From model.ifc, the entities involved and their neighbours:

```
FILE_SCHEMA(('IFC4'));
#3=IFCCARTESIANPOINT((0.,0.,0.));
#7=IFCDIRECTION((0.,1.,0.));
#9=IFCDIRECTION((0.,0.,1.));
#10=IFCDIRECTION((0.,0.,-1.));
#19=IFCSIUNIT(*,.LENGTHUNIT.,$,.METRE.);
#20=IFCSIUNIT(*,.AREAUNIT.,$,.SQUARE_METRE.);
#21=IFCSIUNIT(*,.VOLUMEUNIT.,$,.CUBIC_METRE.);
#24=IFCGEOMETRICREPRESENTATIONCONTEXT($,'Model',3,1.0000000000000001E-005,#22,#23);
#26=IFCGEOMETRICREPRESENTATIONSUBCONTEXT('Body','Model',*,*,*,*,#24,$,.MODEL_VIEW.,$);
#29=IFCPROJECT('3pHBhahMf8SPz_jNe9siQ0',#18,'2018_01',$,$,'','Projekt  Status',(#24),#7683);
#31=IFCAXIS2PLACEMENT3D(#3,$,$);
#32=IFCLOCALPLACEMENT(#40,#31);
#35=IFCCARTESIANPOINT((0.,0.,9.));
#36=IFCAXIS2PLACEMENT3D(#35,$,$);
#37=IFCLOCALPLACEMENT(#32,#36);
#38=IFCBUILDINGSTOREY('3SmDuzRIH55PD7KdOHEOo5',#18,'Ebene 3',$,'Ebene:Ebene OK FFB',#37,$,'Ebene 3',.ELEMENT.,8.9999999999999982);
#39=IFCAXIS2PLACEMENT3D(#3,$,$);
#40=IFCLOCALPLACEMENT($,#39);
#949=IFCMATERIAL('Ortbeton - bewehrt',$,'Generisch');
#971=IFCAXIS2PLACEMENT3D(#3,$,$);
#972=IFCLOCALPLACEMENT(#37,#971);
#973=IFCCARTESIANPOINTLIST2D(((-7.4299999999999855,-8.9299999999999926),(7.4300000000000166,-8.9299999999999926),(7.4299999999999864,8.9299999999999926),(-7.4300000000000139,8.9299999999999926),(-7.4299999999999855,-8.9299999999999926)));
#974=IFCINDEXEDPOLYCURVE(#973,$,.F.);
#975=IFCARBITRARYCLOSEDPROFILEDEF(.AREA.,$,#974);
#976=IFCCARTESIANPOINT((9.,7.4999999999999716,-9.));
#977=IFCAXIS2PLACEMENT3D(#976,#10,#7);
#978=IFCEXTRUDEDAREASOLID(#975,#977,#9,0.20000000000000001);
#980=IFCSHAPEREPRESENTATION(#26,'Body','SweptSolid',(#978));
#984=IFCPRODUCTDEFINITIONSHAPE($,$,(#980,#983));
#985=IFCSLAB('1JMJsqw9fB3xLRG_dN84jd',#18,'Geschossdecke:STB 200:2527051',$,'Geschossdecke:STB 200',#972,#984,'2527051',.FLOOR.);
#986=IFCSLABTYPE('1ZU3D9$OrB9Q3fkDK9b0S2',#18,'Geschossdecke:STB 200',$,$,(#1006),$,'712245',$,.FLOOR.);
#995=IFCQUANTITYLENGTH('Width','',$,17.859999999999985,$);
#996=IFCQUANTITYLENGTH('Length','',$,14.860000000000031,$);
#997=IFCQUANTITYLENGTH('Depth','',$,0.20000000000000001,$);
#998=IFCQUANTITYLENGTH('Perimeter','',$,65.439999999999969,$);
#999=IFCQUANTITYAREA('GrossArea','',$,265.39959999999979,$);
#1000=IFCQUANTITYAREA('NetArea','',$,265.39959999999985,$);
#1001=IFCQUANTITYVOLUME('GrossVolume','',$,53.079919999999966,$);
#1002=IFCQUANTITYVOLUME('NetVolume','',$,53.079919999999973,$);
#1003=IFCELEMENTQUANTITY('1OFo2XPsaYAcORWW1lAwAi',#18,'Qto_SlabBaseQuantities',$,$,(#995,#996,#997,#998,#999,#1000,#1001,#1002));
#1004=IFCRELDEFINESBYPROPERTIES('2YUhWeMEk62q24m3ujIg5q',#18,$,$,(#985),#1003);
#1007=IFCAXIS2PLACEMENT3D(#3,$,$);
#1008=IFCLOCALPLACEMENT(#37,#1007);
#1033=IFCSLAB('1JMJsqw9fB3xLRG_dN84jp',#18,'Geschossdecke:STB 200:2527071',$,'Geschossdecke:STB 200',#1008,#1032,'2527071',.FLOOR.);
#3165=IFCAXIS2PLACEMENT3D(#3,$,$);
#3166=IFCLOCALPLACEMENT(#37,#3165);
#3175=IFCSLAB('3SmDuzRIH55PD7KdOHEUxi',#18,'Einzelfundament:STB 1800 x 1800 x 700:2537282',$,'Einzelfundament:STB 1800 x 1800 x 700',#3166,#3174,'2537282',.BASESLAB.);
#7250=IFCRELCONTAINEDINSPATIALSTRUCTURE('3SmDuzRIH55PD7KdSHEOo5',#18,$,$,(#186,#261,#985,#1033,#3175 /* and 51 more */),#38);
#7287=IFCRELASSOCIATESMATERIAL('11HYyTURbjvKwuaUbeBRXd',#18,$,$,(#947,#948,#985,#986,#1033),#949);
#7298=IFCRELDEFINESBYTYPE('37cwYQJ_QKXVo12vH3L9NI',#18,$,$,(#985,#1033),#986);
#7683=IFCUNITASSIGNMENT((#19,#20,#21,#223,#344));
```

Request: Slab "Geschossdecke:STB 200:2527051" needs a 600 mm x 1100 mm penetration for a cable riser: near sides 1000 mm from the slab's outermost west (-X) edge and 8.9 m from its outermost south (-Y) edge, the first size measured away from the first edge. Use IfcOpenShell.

```python
import numpy as np
import ifcopenshell
import ifcopenshell.api.feature
import ifcopenshell.api.geometry
import ifcopenshell.api.pset
import ifcopenshell.api.root
import ifcopenshell.geom
import ifcopenshell.util.element
import ifcopenshell.util.placement
import ifcopenshell.util.representation
import ifcopenshell.util.shape
import ifcopenshell.util.unit

model = ifcopenshell.open("model.ifc")
unit_scale = ifcopenshell.util.unit.calculate_unit_scale(model)
area_scale = ifcopenshell.util.unit.calculate_unit_scale(model, "AREAUNIT")
volume_scale = ifcopenshell.util.unit.calculate_unit_scale(model, "VOLUMEUNIT")
settings = ifcopenshell.geom.settings()


def volume(element):
    """Net volume in cubic metres, openings subtracted."""
    shape = ifcopenshell.geom.create_shape(settings, element)
    return ifcopenshell.util.shape.get_volume(shape.geometry)


slab = model.by_id(985)
before = volume(slab)

# Extent in the slab's own axes, in metres. The edges named are its -X and -Y sides.
slab_shape = ifcopenshell.geom.create_shape(settings, slab)
vertices = ifcopenshell.util.shape.get_vertices(slab_shape.geometry)
x_min, y_min, bottom = vertices.min(axis=0)
top = vertices[:, 2].max()

opening = ifcopenshell.api.root.create_entity(model, ifc_class="IfcOpeningElement", name="Cable riser opening", predefined_type="OPENING")
context = ifcopenshell.util.representation.get_context(model, "Model", "Body", "MODEL_VIEW")
width, depth = 0.6, 1.1
outline = [(0.0, 0.0), (width, 0.0), (width, depth), (0.0, depth), (0.0, 0.0)]
# Overshoot both faces by 50 mm so the cut is clean.
shape = ifcopenshell.api.geometry.add_slab_representation(
    model, context=context, depth=top - bottom + 0.1, polyline=outline
)
ifcopenshell.api.geometry.assign_representation(model, product=opening, representation=shape)

matrix = ifcopenshell.util.placement.get_local_placement(slab.ObjectPlacement)
matrix[:, 3] = matrix @ np.append(np.array([x_min + 1, y_min + 8.9, bottom - 0.05]) / unit_scale, 1.0)
ifcopenshell.api.geometry.edit_object_placement(model, product=opening, matrix=matrix, is_si=False)
ifcopenshell.api.feature.add_feature(model, feature=opening, element=slab)

after = volume(slab)

# Update the slab's stored quantities.
qto = model.by_id(ifcopenshell.util.element.get_pset(slab, "Qto_SlabBaseQuantities", should_inherit=False)["id"])
ifcopenshell.api.pset.edit_qto(model, qto=qto, properties={
    "NetArea": after / (top - bottom) / area_scale,
    "NetVolume": after / volume_scale,
})

print(f"slab volume {before:.3f} -> {after:.3f} m3")

model.write("model-out.ifc")
```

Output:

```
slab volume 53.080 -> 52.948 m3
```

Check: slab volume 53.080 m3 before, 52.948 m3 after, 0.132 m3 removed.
